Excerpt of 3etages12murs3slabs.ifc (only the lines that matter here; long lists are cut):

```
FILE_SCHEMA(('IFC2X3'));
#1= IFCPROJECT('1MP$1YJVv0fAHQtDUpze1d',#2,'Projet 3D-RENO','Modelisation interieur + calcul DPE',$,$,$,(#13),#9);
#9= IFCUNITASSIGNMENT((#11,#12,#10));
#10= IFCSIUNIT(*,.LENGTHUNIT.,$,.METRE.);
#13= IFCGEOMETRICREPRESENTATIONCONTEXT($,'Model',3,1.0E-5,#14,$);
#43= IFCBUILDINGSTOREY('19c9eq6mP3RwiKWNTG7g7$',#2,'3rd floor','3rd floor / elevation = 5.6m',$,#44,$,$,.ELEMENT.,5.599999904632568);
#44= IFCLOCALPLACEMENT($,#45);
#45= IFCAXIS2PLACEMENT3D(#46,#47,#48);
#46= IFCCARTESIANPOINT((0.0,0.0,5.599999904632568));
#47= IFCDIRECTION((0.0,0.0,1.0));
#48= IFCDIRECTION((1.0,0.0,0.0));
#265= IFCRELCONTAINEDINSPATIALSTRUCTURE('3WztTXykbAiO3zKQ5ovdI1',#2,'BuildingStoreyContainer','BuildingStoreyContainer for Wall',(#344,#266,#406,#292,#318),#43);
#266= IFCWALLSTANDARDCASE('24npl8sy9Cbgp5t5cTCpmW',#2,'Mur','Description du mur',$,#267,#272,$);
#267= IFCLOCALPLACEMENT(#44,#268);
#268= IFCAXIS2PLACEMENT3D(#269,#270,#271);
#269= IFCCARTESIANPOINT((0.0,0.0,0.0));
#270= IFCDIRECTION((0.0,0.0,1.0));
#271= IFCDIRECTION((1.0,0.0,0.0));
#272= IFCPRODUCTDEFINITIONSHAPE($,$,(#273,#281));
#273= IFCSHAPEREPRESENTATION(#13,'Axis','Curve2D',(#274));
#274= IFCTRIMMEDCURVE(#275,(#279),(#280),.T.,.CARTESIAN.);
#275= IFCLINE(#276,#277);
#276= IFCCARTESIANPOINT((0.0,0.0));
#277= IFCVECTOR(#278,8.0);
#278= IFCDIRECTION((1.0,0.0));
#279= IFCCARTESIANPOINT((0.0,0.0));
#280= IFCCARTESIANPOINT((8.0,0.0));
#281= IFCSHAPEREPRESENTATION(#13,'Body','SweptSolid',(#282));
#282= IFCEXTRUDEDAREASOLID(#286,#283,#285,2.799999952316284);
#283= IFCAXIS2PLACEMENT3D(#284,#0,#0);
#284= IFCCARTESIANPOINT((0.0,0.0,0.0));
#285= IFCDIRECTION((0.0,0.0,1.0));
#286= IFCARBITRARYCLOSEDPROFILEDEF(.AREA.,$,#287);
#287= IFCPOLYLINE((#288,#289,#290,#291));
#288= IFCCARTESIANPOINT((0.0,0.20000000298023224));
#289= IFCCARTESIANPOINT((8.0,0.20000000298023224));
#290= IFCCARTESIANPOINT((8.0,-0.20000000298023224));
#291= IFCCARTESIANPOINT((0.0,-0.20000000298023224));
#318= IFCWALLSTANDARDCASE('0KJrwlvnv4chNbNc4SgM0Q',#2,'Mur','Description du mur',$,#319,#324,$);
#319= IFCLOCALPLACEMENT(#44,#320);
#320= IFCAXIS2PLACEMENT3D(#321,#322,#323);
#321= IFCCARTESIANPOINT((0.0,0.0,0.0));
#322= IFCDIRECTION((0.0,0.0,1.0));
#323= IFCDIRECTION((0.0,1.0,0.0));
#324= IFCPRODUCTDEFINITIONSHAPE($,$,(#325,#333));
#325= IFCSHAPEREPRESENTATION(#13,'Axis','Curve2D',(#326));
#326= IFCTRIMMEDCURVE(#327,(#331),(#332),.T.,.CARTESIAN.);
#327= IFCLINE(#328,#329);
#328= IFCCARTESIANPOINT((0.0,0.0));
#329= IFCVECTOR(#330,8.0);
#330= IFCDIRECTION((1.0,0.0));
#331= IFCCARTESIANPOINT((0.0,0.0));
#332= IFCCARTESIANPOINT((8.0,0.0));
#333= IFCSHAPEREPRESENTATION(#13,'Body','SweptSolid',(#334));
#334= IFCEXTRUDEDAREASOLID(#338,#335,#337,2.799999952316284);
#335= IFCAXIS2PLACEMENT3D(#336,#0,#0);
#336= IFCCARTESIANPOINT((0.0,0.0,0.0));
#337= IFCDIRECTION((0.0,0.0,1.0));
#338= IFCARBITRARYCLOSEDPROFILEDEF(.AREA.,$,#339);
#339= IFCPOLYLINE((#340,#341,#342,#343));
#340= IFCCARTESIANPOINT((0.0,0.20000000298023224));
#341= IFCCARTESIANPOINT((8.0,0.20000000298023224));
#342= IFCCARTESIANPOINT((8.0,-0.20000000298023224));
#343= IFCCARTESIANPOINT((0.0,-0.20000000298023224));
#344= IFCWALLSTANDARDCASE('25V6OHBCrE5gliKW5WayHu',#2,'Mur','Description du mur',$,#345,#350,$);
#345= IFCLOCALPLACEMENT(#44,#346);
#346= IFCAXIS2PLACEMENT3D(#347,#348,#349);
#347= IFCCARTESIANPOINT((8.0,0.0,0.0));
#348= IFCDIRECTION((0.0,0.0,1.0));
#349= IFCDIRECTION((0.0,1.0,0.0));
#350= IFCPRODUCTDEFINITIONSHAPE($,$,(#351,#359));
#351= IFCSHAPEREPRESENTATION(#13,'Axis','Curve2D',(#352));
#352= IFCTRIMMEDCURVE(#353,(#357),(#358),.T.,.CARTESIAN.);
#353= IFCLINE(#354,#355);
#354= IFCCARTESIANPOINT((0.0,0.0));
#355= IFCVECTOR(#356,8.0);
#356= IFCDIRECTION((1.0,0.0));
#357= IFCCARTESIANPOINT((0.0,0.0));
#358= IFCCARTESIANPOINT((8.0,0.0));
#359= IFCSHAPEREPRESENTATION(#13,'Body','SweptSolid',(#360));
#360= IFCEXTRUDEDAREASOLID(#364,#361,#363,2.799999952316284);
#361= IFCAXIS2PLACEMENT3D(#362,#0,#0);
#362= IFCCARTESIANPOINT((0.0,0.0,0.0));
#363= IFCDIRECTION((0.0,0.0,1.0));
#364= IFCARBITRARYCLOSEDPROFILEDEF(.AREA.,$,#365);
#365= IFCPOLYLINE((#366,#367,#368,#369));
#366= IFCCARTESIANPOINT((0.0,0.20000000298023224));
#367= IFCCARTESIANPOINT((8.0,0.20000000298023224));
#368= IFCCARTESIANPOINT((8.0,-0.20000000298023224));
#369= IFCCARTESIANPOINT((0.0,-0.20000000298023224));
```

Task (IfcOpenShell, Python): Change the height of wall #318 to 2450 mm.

```python
import ifcopenshell
import ifcopenshell.geom
import ifcopenshell.util.shape

model = ifcopenshell.open("3etages12murs3slabs.ifc")
settings = ifcopenshell.geom.settings()


def volume(element):
    """Net volume in cubic metres, openings subtracted."""
    shape = ifcopenshell.geom.create_shape(settings, element)
    return ifcopenshell.util.shape.get_volume(shape.geometry)


wall = model.by_guid("0KJrwlvnv4chNbNc4SgM0Q")
before = volume(wall)

body = next(r for r in wall.Representation.Representations if r.RepresentationIdentifier == "Body")
solid = body.Items[0]
old_height = solid.Depth
solid.Depth = 2.45
after = volume(wall)

print(f"height {old_height:g} -> {solid.Depth:g}, volume {before:.3f} -> {after:.3f} m3")

model.write("3etages12murs3slabs_rev.ifc")
```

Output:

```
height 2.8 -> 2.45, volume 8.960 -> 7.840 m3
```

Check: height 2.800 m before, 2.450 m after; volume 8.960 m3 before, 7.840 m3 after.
